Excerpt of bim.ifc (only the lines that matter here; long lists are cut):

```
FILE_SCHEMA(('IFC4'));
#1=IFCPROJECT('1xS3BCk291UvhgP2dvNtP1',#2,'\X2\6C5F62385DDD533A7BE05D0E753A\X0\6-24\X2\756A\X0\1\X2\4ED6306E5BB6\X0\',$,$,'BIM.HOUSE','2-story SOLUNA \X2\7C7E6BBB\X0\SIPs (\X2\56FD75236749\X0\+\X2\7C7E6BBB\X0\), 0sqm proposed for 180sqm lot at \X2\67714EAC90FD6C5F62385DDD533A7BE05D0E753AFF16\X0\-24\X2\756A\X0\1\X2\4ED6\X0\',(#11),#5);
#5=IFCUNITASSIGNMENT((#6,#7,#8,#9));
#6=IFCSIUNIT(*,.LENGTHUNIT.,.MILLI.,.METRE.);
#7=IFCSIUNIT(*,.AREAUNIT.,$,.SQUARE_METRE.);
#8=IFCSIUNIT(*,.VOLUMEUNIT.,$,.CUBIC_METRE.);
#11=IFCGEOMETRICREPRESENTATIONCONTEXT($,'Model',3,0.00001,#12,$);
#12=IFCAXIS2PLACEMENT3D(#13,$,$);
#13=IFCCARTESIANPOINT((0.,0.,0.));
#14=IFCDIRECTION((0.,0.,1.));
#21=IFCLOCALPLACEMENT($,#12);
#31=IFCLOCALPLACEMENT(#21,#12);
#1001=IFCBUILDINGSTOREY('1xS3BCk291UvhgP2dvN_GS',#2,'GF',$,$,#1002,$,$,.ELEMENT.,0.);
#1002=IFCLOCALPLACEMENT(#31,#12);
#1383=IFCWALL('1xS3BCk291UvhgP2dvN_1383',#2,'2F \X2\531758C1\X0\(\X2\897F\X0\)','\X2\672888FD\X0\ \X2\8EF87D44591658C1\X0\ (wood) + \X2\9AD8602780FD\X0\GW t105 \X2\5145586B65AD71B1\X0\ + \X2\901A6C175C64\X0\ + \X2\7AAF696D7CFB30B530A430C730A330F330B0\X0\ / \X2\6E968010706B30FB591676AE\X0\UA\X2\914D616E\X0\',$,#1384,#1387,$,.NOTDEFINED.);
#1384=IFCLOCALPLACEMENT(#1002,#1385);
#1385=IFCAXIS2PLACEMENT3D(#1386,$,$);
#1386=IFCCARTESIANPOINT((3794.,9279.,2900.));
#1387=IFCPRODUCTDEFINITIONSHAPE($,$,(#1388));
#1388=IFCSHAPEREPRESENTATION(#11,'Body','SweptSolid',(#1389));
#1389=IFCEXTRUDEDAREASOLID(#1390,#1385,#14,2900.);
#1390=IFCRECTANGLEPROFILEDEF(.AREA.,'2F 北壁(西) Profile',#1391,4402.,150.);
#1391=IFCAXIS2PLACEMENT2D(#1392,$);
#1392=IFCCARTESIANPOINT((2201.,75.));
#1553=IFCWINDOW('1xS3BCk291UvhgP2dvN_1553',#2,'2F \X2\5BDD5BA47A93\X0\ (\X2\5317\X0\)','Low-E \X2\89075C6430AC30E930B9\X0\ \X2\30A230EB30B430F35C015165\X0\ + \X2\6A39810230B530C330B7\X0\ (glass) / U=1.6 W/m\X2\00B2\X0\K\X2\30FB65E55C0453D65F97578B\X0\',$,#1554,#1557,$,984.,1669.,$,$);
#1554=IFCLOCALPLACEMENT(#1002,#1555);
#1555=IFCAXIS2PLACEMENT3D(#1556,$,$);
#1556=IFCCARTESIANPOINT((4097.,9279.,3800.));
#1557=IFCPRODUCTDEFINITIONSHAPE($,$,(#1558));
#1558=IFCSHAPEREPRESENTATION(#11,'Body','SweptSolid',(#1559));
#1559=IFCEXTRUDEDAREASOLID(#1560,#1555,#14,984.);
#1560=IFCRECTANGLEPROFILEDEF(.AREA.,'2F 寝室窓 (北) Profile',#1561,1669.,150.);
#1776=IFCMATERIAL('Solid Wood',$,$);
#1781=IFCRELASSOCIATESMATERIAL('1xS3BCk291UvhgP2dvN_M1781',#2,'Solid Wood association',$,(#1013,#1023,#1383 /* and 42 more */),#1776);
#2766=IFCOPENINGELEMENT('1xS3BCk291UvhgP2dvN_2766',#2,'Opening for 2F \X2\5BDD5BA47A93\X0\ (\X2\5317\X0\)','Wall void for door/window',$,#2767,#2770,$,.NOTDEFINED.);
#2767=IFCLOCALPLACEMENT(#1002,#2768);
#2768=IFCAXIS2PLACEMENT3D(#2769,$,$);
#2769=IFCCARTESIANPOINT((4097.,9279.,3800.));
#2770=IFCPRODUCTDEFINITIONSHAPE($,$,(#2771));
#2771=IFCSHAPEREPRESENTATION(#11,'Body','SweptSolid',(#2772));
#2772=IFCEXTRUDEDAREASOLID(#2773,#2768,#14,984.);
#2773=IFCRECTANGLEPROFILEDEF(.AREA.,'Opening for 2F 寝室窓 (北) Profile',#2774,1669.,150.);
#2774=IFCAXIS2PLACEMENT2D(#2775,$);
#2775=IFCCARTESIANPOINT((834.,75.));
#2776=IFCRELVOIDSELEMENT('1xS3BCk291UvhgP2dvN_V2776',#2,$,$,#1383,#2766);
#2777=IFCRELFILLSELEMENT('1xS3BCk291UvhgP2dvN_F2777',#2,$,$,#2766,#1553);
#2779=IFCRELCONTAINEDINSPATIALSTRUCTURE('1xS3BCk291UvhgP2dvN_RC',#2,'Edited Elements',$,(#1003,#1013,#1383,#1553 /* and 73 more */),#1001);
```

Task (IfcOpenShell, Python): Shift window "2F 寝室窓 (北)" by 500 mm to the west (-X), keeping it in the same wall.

```python
import ifcopenshell
import ifcopenshell.api.geometry
import ifcopenshell.util.placement

model = ifcopenshell.open("bim.ifc")

window = model.by_guid("1xS3BCk291UvhgP2dvN_1553")
opening = window.FillsVoids[0].RelatingOpeningElement
wall = opening.VoidsElements[0].RelatingBuildingElement

wall_matrix = ifcopenshell.util.placement.get_local_placement(wall.ObjectPlacement)
shift = wall_matrix[:3, 0] * -500.0
before = ifcopenshell.util.placement.get_local_placement(window.ObjectPlacement)[:3, 3].copy()

# The window is not placed relative to its opening, so move both.
for product in (opening, window):
    matrix = ifcopenshell.util.placement.get_local_placement(product.ObjectPlacement)
    matrix[:3, 3] += shift
    ifcopenshell.api.geometry.edit_object_placement(model, product=product, matrix=matrix, is_si=False)

after = ifcopenshell.util.placement.get_local_placement(window.ObjectPlacement)[:3, 3]
print("window moved by", (after - before).round(3) + 0.0)

model.write("bim_updated.ifc")
```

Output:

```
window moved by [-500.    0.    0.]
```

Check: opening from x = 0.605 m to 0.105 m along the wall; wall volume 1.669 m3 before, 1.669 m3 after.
